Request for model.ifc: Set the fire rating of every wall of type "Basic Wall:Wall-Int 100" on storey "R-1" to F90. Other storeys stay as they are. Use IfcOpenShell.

First a look at what the model holds.

```python
import ifcopenshell
import ifcopenshell.util.element

model = ifcopenshell.open("model.ifc")
print(model.schema)
storey = next(s for s in model.by_type("IfcBuildingStorey") if s.Name == "R-1")
walls = [e for e in ifcopenshell.util.element.get_decomposition(storey) if e.is_a("IfcWall")]
seen = {}
for e in walls:
    element_type = ifcopenshell.util.element.get_type(e)
    key = (element_type.Name if element_type != e and element_type else None, ifcopenshell.util.element.get_pset(e, "Pset_WallCommon", "FireRating"))
    seen[key] = seen.get(key, 0) + 1
for (name, value), count in sorted(seen.items(), key=str):
    print(count, "x", name, "|", value)
```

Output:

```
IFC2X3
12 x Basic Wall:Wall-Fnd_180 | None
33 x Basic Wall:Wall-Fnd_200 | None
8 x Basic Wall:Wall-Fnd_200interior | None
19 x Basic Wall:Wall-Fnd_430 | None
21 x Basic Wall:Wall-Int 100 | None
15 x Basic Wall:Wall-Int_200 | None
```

```python
import ifcopenshell
import ifcopenshell.api.pset
import ifcopenshell.util.element

model = ifcopenshell.open("model.ifc")

storey = next(s for s in model.by_type("IfcBuildingStorey") if s.Name == "R-1")
walls = [e for e in ifcopenshell.util.element.get_decomposition(storey) if e.is_a("IfcWall")]

count = 0
for e in walls:
    element_type = ifcopenshell.util.element.get_type(e)
    if element_type in (None, e) or element_type.Name != "Basic Wall:Wall-Int 100":
        continue
    # add_pset returns the element's existing set when there is one.
    pset = ifcopenshell.api.pset.add_pset(model, product=e, name="Pset_WallCommon")
    ifcopenshell.api.pset.edit_pset(model, pset=pset, properties={"FireRating": "F90"})
    count += 1

print(count, "walls updated")

model.write("model_updated.ifc")
```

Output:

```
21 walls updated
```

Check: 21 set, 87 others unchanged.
